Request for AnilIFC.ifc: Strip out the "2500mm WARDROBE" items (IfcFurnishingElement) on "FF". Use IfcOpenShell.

First a look at what the model holds.

```python
import ifcopenshell
import ifcopenshell.util.element

model = ifcopenshell.open("AnilIFC.ifc")
print(model.schema)
storey = next(s for s in model.by_type("IfcBuildingStorey") if s.Name == "FF")
furniture = [e for e in ifcopenshell.util.element.get_decomposition(storey) if e.is_a("IfcFurnishingElement")]
seen = {}
for e in furniture:
    element_type = ifcopenshell.util.element.get_type(e)
    name = element_type.Name if element_type not in (None, e) else None
    seen[name] = seen.get(name, 0) + 1
for name, count in sorted(seen.items(), key=str):
    print(count, "x", name)
```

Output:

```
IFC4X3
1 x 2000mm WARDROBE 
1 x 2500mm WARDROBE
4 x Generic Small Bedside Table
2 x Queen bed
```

```python
import ifcopenshell
import ifcopenshell.api.root
import ifcopenshell.util.element

model = ifcopenshell.open("AnilIFC.ifc")

storey = next(s for s in model.by_type("IfcBuildingStorey") if s.Name == "FF")
furniture = [e for e in ifcopenshell.util.element.get_decomposition(storey) if e.is_a("IfcFurnishingElement")]
targets = [e for e in furniture if (t := ifcopenshell.util.element.get_type(e)) not in (None, e) and t.Name == "2500mm WARDROBE"]

for e in targets:
    ifcopenshell.api.root.remove_product(model, product=e)
print(len(targets), "removed")

model.write("AnilIFC-out.ifc")
```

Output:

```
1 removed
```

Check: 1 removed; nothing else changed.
